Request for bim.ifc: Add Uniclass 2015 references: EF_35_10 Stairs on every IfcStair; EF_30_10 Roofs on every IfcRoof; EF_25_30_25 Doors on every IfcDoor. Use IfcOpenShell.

First a look at what the model holds.

```python
import ifcopenshell

model = ifcopenshell.open("bim.ifc")
print(model.schema)
print("classifications:", [c.Name for c in model.by_type("IfcClassification")])
for ifc_class in ("IfcDoor", "IfcRoof", "IfcStair", "IfcWall", "IfcWindow"):
    print(ifc_class, len(model.by_type(ifc_class)))
```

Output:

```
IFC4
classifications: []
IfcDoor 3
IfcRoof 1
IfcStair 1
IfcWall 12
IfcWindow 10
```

```python
import ifcopenshell
import ifcopenshell.api.classification

model = ifcopenshell.open("bim.ifc")

system = ifcopenshell.api.classification.add_classification(model, classification="Uniclass 2015")

codes = {
    "IfcStair": ("EF_35_10", "Stairs"),
    "IfcRoof": ("EF_30_10", "Roofs"),
    "IfcDoor": ("EF_25_30_25", "Doors"),
}
for ifc_class, (code, name) in codes.items():
    products = model.by_type(ifc_class)
    ifcopenshell.api.classification.add_reference(
        model, products=products, classification=system, identification=code, name=name
    )
    print(code, len(products))

model.write("bim-out.ifc")
```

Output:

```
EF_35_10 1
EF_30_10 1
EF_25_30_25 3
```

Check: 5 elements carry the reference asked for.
